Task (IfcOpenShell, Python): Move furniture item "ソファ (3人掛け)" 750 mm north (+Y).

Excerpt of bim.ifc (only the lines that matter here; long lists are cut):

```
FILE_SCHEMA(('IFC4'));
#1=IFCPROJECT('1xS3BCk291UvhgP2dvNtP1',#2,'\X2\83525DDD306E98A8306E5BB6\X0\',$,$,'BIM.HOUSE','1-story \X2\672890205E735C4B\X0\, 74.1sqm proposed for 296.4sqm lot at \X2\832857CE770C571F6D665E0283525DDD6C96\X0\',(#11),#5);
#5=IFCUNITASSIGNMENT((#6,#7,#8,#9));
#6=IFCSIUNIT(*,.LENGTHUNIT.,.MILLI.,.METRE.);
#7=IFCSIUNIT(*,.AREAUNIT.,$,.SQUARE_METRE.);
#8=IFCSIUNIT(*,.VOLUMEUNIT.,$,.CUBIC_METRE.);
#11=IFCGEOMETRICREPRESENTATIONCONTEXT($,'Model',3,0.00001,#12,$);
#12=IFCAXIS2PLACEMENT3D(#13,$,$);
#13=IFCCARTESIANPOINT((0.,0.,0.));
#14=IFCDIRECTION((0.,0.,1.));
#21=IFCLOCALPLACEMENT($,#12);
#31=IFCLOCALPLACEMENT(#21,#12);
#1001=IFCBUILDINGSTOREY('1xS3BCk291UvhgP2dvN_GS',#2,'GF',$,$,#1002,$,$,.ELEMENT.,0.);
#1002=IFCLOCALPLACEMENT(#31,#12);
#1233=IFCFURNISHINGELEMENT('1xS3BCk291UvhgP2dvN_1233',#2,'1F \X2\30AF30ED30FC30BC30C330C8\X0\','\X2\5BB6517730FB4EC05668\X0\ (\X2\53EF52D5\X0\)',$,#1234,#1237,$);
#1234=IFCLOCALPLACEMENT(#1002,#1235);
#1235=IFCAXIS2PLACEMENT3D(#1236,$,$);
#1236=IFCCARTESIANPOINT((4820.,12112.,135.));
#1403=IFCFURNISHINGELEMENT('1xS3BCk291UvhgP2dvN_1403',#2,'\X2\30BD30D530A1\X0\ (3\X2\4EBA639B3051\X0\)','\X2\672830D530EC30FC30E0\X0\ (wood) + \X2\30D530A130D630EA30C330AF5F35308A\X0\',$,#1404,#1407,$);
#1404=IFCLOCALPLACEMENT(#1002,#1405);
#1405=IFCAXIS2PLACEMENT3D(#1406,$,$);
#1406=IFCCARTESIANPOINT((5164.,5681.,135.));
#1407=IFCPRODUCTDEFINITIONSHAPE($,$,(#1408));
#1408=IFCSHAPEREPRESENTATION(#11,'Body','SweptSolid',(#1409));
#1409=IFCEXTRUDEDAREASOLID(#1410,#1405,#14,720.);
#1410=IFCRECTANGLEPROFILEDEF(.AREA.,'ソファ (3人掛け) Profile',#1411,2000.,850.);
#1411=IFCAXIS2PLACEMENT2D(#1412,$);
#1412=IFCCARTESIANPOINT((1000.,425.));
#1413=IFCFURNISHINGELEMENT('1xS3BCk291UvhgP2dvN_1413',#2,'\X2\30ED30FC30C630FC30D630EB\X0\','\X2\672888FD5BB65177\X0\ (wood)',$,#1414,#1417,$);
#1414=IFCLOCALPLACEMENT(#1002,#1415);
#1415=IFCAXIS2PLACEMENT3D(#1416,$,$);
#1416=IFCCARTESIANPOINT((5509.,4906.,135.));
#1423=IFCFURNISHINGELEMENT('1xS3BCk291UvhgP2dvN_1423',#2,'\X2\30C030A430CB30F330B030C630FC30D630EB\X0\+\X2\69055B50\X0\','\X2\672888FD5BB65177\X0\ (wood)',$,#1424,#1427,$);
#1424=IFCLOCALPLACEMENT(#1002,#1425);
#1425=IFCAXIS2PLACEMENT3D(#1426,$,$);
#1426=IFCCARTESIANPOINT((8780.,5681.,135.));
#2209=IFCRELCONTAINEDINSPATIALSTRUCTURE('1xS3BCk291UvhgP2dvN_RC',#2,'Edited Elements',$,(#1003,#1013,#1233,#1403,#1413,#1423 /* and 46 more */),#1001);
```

```python
import ifcopenshell
import ifcopenshell.api.geometry
import ifcopenshell.util.placement
import ifcopenshell.util.unit

model = ifcopenshell.open("bim.ifc")
unit_scale = ifcopenshell.util.unit.calculate_unit_scale(model)

item = model.by_id(1403)
matrix = ifcopenshell.util.placement.get_local_placement(item.ObjectPlacement)
matrix[1, 3] += 0.75 / unit_scale
ifcopenshell.api.geometry.edit_object_placement(model, product=item, matrix=matrix, is_si=False)

print(ifcopenshell.util.placement.get_local_placement(item.ObjectPlacement).round(3) + 0.0)

model.write("bim_updated.ifc")
```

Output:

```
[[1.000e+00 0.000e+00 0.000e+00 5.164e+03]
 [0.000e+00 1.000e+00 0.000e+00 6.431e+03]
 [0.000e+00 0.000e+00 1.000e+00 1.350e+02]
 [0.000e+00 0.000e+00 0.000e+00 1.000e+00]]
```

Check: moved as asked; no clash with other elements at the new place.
